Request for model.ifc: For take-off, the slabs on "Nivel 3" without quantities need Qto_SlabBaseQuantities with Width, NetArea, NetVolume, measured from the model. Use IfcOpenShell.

First a look at what the model holds.

```python
import ifcopenshell
import ifcopenshell.util.element
import ifcopenshell.util.unit

model = ifcopenshell.open("model.ifc")
print(model.schema)
for unit_type in ("LENGTHUNIT", "AREAUNIT", "VOLUMEUNIT"):
    print(unit_type, ifcopenshell.util.unit.calculate_unit_scale(model, unit_type))
storey = next(s for s in model.by_type("IfcBuildingStorey") if s.Name == "Nivel 3")
slabs = [e for e in ifcopenshell.util.element.get_decomposition(storey) if e.is_a("IfcSlab")]
for e in sorted(slabs, key=lambda e: e.id()):
    print(e.id(), e.is_a(), e.Name, list(ifcopenshell.util.element.get_psets(e, qtos_only=True)), sep=" | ")
```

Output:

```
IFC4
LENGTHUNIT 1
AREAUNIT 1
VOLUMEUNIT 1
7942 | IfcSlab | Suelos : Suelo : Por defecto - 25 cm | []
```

```python
import ifcopenshell
import ifcopenshell.api.pset
import ifcopenshell.geom
import ifcopenshell.util.element
import ifcopenshell.util.shape
import ifcopenshell.util.unit

model = ifcopenshell.open("model.ifc")
unit_scale = ifcopenshell.util.unit.calculate_unit_scale(model)
area_scale = ifcopenshell.util.unit.calculate_unit_scale(model, "AREAUNIT")
volume_scale = ifcopenshell.util.unit.calculate_unit_scale(model, "VOLUMEUNIT")
settings = ifcopenshell.geom.settings()

storey = next(s for s in model.by_type("IfcBuildingStorey") if s.Name == "Nivel 3")
slabs = [e for e in ifcopenshell.util.element.get_decomposition(storey) if e.is_a("IfcSlab")]

for e in sorted(slabs, key=lambda e: e.id()):
    if ifcopenshell.util.element.get_psets(e, qtos_only=True, should_inherit=False):
        continue
    # Geometry comes back in metres, in the element's own axes.
    shape = ifcopenshell.geom.create_shape(settings, e)
    values = {
        "Width": ifcopenshell.util.shape.get_z(shape.geometry) / unit_scale,
        "NetArea": ifcopenshell.util.shape.get_footprint_area(shape.geometry) / area_scale,
        "NetVolume": ifcopenshell.util.shape.get_volume(shape.geometry) / volume_scale,
    }
    qto = ifcopenshell.api.pset.add_qto(model, product=e, name="Qto_SlabBaseQuantities")
    ifcopenshell.api.pset.edit_qto(model, qto=qto, properties=values)
    print(e.id(), {k: round(v, 3) for k, v in values.items()})

model.write("model_rev.ifc")
```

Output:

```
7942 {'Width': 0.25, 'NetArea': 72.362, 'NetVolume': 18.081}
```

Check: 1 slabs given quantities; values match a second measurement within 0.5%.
